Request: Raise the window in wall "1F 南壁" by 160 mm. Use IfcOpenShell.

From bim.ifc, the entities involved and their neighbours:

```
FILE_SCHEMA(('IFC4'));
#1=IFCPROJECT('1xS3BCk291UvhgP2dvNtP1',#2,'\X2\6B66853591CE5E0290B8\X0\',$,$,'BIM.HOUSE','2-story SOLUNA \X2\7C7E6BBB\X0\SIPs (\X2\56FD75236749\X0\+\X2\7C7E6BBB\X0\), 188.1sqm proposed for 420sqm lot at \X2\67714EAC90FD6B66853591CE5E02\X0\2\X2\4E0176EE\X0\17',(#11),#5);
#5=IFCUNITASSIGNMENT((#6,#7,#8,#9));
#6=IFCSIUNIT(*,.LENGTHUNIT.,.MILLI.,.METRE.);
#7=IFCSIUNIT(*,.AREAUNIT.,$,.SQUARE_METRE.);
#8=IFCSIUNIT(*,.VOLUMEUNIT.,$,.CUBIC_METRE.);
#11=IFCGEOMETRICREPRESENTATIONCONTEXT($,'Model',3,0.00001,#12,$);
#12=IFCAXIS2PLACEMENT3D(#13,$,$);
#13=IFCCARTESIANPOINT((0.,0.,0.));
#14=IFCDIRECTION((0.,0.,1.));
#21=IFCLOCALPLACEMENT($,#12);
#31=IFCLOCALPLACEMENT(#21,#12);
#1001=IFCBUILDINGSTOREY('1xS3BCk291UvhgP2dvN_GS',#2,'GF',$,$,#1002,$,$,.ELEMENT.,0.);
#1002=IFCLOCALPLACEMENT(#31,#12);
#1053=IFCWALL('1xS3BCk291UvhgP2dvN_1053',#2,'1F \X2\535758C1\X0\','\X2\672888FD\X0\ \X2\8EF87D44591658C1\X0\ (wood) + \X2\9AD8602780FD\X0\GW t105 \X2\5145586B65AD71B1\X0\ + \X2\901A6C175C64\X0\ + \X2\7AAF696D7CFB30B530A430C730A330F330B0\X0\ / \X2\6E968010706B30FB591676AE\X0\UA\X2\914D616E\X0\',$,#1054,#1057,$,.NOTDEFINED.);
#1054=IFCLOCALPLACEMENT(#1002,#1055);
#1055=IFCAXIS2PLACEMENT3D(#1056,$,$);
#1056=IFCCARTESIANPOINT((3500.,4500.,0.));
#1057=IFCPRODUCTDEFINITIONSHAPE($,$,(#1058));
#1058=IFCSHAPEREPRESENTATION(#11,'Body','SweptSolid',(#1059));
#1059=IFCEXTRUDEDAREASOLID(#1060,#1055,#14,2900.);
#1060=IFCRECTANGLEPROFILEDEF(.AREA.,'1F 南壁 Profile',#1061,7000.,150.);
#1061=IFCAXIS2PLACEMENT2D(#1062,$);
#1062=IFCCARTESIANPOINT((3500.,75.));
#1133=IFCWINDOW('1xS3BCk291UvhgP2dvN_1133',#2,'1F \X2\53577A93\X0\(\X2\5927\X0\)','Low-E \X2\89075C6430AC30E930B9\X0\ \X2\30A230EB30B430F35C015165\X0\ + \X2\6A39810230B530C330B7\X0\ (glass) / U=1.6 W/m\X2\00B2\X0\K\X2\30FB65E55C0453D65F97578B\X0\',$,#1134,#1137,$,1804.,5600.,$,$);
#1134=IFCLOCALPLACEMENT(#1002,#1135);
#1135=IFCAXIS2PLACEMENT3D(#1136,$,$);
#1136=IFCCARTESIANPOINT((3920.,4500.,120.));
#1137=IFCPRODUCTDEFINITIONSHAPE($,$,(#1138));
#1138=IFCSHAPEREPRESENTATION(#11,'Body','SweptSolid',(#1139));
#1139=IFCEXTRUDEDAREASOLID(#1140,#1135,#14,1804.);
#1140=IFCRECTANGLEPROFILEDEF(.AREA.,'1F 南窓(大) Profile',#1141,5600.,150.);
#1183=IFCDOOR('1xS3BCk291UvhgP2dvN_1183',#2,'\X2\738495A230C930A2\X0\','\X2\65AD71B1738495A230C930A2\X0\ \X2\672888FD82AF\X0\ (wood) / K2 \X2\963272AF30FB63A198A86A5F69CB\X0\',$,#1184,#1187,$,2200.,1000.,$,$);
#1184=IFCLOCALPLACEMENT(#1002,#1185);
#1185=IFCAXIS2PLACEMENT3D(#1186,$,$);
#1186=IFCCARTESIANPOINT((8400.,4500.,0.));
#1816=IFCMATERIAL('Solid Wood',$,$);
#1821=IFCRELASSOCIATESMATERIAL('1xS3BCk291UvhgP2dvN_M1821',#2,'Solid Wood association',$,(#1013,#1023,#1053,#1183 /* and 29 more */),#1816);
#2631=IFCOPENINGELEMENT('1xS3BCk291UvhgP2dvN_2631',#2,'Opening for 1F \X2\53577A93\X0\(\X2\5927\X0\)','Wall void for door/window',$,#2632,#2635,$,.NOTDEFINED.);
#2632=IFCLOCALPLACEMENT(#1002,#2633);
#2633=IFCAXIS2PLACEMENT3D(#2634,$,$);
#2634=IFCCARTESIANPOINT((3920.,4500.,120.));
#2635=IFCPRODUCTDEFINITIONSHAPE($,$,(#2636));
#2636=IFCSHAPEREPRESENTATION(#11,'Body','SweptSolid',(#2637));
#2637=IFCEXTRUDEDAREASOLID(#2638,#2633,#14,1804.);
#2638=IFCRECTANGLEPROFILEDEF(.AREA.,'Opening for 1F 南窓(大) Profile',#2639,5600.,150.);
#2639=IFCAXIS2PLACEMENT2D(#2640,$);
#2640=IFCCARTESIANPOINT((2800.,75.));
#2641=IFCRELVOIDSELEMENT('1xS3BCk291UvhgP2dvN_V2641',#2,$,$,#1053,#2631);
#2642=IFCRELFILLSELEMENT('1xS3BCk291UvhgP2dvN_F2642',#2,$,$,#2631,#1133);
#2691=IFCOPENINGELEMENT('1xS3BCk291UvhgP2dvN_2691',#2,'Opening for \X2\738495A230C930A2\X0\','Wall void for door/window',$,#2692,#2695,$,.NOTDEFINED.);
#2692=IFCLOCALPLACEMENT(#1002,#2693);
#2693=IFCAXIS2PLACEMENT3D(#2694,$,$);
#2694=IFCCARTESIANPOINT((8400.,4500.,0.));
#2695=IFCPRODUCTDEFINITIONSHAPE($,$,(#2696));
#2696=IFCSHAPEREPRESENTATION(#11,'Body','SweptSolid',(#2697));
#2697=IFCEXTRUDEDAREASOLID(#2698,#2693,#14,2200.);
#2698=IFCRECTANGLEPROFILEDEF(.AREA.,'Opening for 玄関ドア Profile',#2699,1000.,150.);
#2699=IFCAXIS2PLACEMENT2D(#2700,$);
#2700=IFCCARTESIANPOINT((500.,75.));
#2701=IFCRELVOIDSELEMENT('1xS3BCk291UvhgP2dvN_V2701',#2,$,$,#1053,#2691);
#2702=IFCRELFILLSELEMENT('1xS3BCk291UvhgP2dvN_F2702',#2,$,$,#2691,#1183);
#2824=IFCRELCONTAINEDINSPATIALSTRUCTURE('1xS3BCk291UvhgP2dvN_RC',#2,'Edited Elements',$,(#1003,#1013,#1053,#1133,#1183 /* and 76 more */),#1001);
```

```python
import numpy as np
import ifcopenshell
import ifcopenshell.api.geometry
import ifcopenshell.util.placement
import ifcopenshell.util.unit

model = ifcopenshell.open("bim.ifc")
unit_scale = ifcopenshell.util.unit.calculate_unit_scale(model)

window = model.by_id(1133)
opening = window.FillsVoids[0].RelatingOpeningElement
dz = 0.16 / unit_scale

shift = np.array([0.0, 0.0, dz])
# The window is not placed relative to its opening, so move both.
for product in (opening, window):
    matrix = ifcopenshell.util.placement.get_local_placement(product.ObjectPlacement)
    matrix[:3, 3] += shift
    ifcopenshell.api.geometry.edit_object_placement(model, product=product, matrix=matrix, is_si=False)

print(f"moved by {dz * unit_scale:+.3f} m")

model.write("bim-out.ifc")
```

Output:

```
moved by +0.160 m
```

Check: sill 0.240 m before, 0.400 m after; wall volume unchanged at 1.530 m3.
